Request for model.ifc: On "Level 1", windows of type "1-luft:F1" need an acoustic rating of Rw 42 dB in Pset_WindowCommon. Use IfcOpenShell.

First a look at what the model holds.

```python
import ifcopenshell
import ifcopenshell.util.element

model = ifcopenshell.open("model.ifc")
print(model.schema)
storey = next(s for s in model.by_type("IfcBuildingStorey") if s.Name == "Level 1")
windows = [e for e in ifcopenshell.util.element.get_decomposition(storey) if e.is_a("IfcWindow")]
seen = {}
for e in windows:
    element_type = ifcopenshell.util.element.get_type(e)
    key = (element_type.Name if element_type != e and element_type else None, ifcopenshell.util.element.get_pset(e, "Pset_WindowCommon", "AcousticRating"))
    seen[key] = seen.get(key, 0) + 1
for (name, value), count in sorted(seen.items(), key=str):
    print(count, "x", name, "|", value)
```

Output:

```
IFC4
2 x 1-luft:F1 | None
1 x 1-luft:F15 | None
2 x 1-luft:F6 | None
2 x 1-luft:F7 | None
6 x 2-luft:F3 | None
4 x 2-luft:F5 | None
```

```python
import ifcopenshell
import ifcopenshell.api.pset
import ifcopenshell.util.element

model = ifcopenshell.open("model.ifc")

storey = next(s for s in model.by_type("IfcBuildingStorey") if s.Name == "Level 1")
windows = [e for e in ifcopenshell.util.element.get_decomposition(storey) if e.is_a("IfcWindow")]

count = 0
for e in windows:
    element_type = ifcopenshell.util.element.get_type(e)
    if element_type in (None, e) or element_type.Name != "1-luft:F1":
        continue
    # add_pset returns the element's existing set when there is one.
    pset = ifcopenshell.api.pset.add_pset(model, product=e, name="Pset_WindowCommon")
    ifcopenshell.api.pset.edit_pset(model, pset=pset, properties={"AcousticRating": "Rw 42 dB"})
    count += 1

print(count, "windows updated")

model.write("model-out.ifc")
```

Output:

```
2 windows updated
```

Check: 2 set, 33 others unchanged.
